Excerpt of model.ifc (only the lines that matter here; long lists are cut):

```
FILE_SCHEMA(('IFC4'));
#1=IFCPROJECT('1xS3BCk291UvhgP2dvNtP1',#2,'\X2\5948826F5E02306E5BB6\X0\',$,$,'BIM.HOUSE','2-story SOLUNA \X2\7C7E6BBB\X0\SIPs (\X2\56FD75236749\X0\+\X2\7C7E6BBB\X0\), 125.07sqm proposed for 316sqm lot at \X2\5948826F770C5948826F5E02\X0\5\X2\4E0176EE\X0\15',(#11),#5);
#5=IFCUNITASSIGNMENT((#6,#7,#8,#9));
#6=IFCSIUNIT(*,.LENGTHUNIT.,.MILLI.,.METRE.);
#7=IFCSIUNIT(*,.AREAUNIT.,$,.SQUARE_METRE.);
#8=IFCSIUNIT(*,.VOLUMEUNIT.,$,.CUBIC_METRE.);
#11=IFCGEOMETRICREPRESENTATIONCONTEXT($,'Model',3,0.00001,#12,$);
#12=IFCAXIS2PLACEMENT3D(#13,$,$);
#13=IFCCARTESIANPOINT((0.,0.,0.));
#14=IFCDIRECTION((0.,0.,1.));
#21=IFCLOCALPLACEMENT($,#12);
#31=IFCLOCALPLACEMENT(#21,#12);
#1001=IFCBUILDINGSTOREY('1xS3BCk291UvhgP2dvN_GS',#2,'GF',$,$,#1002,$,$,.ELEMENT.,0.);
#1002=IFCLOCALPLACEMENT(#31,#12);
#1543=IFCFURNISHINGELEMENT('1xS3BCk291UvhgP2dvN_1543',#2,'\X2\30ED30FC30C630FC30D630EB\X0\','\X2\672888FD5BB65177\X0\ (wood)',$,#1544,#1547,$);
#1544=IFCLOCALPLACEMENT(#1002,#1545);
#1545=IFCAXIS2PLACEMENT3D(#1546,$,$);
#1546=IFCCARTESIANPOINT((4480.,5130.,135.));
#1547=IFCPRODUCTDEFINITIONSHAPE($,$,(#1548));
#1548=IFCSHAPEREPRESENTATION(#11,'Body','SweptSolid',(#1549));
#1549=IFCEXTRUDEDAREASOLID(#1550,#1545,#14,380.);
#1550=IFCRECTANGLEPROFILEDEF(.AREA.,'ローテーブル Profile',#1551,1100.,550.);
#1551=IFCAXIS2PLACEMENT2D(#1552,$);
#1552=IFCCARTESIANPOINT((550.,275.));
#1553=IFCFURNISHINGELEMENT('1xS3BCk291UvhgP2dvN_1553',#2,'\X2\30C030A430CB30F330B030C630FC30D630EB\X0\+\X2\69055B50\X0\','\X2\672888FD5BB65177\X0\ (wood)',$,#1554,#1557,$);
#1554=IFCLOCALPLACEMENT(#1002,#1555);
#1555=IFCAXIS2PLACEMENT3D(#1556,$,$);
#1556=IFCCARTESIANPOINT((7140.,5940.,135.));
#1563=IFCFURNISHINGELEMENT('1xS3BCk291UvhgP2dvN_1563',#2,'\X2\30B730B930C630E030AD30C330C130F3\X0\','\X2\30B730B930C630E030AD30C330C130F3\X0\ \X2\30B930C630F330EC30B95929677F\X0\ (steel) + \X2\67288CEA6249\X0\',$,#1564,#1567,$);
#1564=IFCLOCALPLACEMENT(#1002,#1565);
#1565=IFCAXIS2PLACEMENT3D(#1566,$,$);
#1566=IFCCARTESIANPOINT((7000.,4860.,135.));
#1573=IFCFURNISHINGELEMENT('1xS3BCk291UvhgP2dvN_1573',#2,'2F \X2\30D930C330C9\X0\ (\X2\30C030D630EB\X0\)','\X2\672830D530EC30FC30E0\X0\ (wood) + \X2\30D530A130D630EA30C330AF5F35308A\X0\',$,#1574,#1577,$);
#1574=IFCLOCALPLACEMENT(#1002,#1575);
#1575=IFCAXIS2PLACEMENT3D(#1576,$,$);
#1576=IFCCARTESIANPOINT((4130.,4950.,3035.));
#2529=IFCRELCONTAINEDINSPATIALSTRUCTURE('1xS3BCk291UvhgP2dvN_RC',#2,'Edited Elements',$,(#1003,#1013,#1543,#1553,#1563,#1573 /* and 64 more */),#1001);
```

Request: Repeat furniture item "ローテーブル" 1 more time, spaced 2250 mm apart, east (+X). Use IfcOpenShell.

```python
import numpy as np
import ifcopenshell
import ifcopenshell.api.geometry
import ifcopenshell.api.root
import ifcopenshell.util.element
import ifcopenshell.util.placement
import ifcopenshell.util.unit

model = ifcopenshell.open("model.ifc")
unit_scale = ifcopenshell.util.unit.calculate_unit_scale(model)


def reuse_history(source, copy):
    """copy_class also copies each property set's owner history, people and application; keep the originals."""
    for rel in copy.IsDefinedBy:
        if rel.is_a("IfcRelDefinesByProperties") and (history := rel.RelatingPropertyDefinition.OwnerHistory):
            rel.RelatingPropertyDefinition.OwnerHistory = source.OwnerHistory
            ifcopenshell.util.element.remove_deep2(model, history)


source = model.by_id(1543)
base = ifcopenshell.util.placement.get_local_placement(source.ObjectPlacement)
step = np.array([1.0, 0.0, 0.0]) * 2.25 / unit_scale

for i in range(1, 2):
    copy = ifcopenshell.api.root.copy_class(model, product=source)
    copy.Representation = ifcopenshell.util.element.copy_deep(
        model, source.Representation, exclude=["IfcGeometricRepresentationContext", "IfcRepresentationMap"]
    )
    reuse_history(source, copy)
    matrix = base.copy()
    matrix[:3, 3] += i * step
    print("added at", matrix[:3, 3].round(3) + 0.0)
    ifcopenshell.api.geometry.edit_object_placement(model, product=copy, matrix=matrix, is_si=False)

model.write("model-out.ifc")
```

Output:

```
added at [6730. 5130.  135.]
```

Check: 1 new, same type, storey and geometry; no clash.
